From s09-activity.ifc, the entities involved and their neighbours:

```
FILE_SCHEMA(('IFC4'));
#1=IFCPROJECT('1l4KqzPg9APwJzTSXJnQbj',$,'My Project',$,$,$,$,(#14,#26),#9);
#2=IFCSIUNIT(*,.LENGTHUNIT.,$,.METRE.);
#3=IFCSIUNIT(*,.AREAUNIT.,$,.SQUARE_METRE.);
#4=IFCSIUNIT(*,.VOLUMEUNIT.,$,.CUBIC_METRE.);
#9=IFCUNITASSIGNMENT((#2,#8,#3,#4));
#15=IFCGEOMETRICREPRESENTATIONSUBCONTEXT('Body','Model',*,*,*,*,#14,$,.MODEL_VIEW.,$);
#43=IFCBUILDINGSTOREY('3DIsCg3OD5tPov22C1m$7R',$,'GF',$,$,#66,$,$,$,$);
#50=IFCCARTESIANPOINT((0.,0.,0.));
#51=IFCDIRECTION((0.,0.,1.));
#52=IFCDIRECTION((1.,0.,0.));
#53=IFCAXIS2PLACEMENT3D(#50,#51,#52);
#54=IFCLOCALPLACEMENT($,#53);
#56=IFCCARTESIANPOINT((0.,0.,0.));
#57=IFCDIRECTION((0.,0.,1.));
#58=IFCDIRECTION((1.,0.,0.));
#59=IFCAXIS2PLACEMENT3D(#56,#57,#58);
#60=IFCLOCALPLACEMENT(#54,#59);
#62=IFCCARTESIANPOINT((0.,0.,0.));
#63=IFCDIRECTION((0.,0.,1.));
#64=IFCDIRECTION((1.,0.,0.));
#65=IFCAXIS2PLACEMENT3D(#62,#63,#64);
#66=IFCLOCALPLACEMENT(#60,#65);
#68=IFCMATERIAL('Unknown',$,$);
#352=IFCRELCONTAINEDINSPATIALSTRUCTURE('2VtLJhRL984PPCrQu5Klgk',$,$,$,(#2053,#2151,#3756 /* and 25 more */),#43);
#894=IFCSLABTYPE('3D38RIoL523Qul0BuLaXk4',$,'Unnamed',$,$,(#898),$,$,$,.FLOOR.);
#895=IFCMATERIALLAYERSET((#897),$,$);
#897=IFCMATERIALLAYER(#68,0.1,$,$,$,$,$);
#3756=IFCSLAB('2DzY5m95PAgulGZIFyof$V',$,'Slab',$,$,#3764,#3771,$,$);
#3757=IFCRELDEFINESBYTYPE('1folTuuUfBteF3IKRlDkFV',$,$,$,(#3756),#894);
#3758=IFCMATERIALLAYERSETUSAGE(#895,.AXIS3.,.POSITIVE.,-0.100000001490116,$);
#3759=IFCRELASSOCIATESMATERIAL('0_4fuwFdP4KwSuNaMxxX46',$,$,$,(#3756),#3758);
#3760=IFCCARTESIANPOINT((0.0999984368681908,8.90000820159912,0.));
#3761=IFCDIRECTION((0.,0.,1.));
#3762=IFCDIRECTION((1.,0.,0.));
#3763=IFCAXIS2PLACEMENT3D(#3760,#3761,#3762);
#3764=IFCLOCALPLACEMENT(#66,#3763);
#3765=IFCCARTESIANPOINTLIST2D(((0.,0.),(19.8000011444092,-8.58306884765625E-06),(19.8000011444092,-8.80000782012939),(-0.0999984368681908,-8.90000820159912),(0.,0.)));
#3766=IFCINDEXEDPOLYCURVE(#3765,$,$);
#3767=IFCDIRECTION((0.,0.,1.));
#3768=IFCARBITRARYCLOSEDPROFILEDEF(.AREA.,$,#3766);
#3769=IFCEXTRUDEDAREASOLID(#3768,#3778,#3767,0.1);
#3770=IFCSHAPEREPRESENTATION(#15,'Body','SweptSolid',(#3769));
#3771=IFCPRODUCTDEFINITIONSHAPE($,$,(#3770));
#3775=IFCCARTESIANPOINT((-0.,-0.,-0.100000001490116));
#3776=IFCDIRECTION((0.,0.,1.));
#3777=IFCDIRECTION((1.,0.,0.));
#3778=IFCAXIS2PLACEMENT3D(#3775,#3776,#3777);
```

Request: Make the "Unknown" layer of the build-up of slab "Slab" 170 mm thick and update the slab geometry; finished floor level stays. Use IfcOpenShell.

```python
import ifcopenshell
import ifcopenshell.util.element
import ifcopenshell.util.representation
import ifcopenshell.util.unit

model = ifcopenshell.open("s09-activity.ifc")
unit_scale = ifcopenshell.util.unit.calculate_unit_scale(model)

layer_set = model.by_id(895)
layer = next(l for l in layer_set.MaterialLayers if l.Material and l.Material.Name == "Unknown")
change = 0.17 / unit_scale - layer.LayerThickness
layer.LayerThickness += change

# Geometry does not follow the layer set by itself.
slabs = [e for e in ifcopenshell.util.element.get_elements_by_material(model, layer_set) if e.is_a("IfcSlab")]
for slab in sorted(slabs, key=lambda e: e.id()):
    body = ifcopenshell.util.representation.get_representation(slab, "Model", "Body")
    solid = body.Items[0]
    old_depth = solid.Depth
    solid.Depth += change
    # Extruded upwards: lower the start of the extrusion so the top stays.
    x, y, z = solid.Position.Location.Coordinates
    solid.Position.Location = model.createIfcCartesianPoint((x, y, z - change))
    print(slab.id(), f"{old_depth:g} -> {solid.Depth:g}")

# The layers are counted up from the underside, which has moved.
for usage in {ifcopenshell.util.element.get_material(slab) for slab in slabs}:
    usage.OffsetFromReferenceLine -= change

model.write("s09-activity_rev.ifc")
```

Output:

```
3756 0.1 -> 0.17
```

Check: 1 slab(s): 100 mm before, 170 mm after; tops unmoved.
